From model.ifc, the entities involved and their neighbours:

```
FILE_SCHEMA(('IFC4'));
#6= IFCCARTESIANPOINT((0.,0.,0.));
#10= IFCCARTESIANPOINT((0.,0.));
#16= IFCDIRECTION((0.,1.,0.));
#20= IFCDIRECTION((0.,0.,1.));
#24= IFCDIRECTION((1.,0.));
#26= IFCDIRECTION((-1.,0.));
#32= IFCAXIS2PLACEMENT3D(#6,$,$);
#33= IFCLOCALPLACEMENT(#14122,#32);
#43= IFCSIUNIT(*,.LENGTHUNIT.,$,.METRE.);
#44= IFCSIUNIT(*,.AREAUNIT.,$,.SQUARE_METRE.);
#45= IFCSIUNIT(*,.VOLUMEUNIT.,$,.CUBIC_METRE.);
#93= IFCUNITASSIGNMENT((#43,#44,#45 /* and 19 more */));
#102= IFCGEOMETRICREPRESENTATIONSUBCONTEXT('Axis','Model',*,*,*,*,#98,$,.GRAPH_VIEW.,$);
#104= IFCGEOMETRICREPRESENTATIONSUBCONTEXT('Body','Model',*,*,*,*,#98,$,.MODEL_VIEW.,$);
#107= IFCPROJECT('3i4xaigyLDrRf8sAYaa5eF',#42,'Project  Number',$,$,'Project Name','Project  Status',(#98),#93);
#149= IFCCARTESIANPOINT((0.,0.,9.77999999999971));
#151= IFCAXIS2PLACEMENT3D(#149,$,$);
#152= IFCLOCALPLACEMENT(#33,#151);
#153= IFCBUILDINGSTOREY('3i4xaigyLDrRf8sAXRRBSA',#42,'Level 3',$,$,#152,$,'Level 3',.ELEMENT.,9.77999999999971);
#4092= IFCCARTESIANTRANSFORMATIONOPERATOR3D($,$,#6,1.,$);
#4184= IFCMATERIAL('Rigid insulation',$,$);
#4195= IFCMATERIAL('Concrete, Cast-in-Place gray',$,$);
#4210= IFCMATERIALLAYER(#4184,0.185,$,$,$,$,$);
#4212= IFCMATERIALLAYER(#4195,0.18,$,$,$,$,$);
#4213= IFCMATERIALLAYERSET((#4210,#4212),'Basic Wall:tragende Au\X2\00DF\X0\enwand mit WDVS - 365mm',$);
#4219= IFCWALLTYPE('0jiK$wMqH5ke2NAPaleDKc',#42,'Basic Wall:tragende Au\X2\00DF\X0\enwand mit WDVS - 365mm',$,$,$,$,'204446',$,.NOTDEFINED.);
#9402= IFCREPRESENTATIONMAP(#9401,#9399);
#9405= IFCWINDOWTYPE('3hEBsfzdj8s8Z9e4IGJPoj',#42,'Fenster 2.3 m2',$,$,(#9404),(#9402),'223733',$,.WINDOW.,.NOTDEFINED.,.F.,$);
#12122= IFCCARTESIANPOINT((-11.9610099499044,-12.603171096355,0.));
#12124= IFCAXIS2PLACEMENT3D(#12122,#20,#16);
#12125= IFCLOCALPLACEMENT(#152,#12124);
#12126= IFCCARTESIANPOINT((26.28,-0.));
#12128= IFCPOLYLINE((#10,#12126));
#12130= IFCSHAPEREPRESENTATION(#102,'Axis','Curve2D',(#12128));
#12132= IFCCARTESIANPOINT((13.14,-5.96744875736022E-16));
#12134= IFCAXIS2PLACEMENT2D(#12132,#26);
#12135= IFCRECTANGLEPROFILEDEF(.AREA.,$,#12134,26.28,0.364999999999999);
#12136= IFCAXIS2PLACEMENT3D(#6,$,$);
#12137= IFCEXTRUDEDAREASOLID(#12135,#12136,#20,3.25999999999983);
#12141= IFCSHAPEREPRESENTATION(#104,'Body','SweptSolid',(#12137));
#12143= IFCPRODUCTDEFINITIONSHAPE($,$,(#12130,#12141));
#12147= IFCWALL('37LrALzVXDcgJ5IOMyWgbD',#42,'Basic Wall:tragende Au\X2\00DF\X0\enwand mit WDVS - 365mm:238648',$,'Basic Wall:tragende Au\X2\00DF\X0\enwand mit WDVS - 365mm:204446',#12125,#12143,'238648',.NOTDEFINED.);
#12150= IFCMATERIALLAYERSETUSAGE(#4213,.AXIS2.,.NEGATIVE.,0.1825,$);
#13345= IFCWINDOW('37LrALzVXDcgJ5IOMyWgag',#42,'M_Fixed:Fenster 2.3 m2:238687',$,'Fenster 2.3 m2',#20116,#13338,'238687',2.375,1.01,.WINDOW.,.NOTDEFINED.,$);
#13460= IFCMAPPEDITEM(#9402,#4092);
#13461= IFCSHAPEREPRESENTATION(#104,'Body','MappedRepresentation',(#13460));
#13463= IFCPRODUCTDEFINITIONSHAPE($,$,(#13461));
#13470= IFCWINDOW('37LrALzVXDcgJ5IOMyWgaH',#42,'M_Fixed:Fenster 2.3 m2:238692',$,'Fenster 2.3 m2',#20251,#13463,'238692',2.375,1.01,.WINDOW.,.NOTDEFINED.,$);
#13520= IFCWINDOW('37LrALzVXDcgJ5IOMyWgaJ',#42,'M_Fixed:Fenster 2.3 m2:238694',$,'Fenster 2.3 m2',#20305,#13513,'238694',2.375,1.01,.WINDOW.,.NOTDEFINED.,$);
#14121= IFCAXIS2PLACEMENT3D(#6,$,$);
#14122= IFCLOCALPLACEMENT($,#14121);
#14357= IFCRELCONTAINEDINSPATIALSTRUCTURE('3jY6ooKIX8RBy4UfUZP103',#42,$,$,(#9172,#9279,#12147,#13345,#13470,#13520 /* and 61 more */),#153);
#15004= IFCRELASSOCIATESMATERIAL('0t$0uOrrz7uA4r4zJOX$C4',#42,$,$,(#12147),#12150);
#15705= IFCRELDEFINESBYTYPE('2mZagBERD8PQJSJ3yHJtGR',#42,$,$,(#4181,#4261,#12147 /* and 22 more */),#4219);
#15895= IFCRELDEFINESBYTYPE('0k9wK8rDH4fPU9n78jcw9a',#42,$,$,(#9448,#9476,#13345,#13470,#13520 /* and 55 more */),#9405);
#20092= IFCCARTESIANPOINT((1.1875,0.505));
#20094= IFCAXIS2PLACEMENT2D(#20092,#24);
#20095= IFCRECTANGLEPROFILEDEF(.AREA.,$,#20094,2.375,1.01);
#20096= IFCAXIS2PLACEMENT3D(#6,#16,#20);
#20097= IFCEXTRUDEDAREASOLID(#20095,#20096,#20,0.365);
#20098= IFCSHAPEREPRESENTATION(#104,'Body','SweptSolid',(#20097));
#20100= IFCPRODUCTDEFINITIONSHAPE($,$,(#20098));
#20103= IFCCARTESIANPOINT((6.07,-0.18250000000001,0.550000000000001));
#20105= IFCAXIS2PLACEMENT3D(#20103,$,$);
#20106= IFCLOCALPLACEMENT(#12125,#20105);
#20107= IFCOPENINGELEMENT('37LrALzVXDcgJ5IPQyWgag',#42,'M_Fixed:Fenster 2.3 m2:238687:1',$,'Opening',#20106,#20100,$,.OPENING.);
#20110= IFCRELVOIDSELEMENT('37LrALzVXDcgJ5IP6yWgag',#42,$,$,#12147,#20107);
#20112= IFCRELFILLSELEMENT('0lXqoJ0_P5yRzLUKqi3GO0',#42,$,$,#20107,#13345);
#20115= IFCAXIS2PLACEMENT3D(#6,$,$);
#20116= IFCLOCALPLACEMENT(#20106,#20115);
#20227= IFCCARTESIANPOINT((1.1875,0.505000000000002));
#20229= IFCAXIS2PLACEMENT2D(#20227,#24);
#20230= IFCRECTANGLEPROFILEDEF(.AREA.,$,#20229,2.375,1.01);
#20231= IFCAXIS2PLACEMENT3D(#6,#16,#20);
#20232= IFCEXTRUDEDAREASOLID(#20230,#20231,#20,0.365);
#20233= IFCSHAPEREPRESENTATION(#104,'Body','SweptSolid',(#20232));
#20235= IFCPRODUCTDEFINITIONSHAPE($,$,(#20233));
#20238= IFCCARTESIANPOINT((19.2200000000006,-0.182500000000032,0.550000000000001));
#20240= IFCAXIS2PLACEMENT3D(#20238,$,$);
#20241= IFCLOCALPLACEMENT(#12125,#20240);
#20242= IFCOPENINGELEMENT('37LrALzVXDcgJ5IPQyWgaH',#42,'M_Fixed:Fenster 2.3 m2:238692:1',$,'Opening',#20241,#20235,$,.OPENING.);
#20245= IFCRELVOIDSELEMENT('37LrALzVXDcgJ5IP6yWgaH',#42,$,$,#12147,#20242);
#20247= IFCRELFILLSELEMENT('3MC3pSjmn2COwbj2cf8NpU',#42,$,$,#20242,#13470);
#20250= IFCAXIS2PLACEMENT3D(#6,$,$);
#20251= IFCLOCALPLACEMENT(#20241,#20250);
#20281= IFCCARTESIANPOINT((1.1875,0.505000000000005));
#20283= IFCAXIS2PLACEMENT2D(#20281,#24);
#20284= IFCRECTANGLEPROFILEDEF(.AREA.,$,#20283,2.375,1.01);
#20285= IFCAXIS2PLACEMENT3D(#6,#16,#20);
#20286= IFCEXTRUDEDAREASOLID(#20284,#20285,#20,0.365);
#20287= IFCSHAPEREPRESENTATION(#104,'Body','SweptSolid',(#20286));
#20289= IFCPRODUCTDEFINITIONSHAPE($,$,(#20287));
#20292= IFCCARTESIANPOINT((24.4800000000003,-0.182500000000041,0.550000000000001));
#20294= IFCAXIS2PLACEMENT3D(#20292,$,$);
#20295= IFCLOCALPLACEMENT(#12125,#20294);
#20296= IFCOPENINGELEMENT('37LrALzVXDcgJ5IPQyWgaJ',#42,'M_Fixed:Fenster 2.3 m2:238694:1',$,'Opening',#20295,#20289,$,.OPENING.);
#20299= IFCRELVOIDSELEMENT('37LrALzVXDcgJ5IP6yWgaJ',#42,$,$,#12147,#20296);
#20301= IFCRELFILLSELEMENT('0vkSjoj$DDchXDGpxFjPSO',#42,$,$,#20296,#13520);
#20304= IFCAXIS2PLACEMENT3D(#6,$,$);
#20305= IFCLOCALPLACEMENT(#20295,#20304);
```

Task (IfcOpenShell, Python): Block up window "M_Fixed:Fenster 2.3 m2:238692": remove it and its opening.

```python
import ifcopenshell
import ifcopenshell.api.feature
import ifcopenshell.api.root
import ifcopenshell.geom
import ifcopenshell.util.shape

model = ifcopenshell.open("model.ifc")
settings = ifcopenshell.geom.settings()


def volume(element):
    """Net volume in cubic metres, openings subtracted."""
    shape = ifcopenshell.geom.create_shape(settings, element)
    return ifcopenshell.util.shape.get_volume(shape.geometry)


window = model.by_guid("37LrALzVXDcgJ5IOMyWgaH")
opening = window.FillsVoids[0].RelatingOpeningElement
wall = opening.VoidsElements[0].RelatingBuildingElement
before = volume(wall)

ifcopenshell.api.root.remove_product(model, product=window)
ifcopenshell.api.feature.remove_feature(model, feature=opening)

after = volume(wall)

print(f"wall volume {before:.3f} -> {after:.3f} m3")

model.write("model-out.ifc")
```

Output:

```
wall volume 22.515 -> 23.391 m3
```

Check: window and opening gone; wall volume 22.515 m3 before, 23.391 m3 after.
